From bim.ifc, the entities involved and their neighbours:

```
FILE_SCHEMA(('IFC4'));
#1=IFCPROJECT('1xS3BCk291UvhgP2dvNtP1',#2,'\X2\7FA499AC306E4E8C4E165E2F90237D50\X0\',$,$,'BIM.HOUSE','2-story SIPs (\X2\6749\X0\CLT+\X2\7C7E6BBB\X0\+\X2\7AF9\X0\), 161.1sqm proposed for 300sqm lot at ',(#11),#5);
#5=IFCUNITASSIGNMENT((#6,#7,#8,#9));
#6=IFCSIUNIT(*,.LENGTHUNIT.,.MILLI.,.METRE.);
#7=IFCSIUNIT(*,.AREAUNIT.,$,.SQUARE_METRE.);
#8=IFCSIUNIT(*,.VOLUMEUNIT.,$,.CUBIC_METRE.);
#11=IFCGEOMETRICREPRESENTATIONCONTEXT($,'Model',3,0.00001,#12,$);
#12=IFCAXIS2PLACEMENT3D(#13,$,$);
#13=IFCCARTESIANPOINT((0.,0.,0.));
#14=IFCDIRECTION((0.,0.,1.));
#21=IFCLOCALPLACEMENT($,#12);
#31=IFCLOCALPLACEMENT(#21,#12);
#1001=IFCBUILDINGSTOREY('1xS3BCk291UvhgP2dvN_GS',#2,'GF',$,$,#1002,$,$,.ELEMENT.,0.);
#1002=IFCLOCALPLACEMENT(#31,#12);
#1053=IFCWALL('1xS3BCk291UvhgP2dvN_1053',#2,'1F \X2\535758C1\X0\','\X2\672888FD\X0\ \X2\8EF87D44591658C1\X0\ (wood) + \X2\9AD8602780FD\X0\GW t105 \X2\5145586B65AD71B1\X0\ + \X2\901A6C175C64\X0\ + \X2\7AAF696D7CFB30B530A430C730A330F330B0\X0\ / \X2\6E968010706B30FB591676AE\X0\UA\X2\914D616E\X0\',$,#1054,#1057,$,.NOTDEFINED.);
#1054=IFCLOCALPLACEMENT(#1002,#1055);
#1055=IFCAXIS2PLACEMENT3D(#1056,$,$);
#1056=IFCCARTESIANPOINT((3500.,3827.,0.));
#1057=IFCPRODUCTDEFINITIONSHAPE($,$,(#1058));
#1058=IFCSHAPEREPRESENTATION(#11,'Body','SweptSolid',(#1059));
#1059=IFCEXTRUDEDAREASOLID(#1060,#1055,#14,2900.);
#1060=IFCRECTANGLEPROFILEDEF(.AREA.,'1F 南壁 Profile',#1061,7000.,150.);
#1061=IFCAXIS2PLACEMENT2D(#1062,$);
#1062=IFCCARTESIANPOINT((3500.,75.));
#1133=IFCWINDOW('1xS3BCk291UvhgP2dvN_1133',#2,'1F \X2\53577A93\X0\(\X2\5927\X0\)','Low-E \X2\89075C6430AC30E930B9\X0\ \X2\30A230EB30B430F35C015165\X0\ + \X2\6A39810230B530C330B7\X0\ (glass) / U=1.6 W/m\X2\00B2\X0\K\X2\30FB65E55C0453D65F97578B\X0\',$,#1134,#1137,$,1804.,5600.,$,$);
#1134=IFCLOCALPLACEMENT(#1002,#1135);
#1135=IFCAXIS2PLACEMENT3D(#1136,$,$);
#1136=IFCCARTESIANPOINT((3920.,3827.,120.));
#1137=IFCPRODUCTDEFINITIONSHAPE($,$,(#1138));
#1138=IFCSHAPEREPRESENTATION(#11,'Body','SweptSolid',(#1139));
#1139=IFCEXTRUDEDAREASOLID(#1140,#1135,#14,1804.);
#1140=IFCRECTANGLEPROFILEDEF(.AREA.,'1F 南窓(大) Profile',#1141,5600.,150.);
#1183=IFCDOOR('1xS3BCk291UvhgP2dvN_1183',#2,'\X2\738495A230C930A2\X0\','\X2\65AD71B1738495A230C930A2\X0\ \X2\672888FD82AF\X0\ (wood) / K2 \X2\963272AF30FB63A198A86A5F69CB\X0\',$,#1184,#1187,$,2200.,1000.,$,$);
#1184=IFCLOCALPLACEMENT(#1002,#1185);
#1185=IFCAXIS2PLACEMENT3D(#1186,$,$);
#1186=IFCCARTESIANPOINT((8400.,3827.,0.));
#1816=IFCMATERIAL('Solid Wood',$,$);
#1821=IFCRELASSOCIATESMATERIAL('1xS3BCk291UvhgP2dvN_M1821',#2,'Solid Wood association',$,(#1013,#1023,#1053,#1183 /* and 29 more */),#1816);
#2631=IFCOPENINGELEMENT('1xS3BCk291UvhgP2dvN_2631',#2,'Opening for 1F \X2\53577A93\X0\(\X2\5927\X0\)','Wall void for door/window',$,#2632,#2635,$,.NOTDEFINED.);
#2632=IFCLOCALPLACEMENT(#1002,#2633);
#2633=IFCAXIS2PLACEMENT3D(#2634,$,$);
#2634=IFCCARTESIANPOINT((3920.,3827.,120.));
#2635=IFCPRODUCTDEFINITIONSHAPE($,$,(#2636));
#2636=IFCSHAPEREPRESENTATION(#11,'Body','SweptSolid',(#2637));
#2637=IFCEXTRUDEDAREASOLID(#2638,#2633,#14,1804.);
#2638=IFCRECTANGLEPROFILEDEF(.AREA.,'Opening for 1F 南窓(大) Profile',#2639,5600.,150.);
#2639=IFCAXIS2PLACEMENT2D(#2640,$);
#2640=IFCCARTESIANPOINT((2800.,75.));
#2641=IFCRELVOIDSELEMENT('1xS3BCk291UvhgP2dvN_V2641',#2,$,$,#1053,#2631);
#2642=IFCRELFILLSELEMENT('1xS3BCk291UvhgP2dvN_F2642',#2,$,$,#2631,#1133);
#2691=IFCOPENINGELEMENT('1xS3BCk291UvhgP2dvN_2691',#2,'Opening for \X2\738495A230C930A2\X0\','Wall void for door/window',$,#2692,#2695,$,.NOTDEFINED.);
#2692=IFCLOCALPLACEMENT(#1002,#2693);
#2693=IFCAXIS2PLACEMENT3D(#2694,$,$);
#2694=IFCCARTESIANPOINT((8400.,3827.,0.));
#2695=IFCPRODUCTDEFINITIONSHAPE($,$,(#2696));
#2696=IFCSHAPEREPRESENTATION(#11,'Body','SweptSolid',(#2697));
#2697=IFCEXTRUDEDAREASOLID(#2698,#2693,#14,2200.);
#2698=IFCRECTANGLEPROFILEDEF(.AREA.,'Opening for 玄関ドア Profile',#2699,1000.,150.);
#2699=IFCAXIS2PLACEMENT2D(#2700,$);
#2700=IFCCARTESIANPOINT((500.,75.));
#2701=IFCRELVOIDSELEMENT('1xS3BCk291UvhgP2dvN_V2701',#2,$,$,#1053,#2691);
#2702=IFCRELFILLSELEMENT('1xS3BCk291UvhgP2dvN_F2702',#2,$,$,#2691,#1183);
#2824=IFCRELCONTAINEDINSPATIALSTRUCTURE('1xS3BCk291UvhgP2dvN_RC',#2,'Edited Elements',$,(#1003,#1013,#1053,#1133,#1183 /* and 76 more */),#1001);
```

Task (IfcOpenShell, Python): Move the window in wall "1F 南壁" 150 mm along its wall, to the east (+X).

```python
import ifcopenshell
import ifcopenshell.api.geometry
import ifcopenshell.util.placement
import ifcopenshell.util.unit

model = ifcopenshell.open("bim.ifc")
unit_scale = ifcopenshell.util.unit.calculate_unit_scale(model)

window = model.by_guid("1xS3BCk291UvhgP2dvN_1133")
opening = window.FillsVoids[0].RelatingOpeningElement
wall = opening.VoidsElements[0].RelatingBuildingElement

wall_matrix = ifcopenshell.util.placement.get_local_placement(wall.ObjectPlacement)
shift = wall_matrix[:3, 0] * 0.15 / unit_scale
before = ifcopenshell.util.placement.get_local_placement(window.ObjectPlacement)[:3, 3].copy()

# The window is not placed relative to its opening, so move both.
for product in (opening, window):
    matrix = ifcopenshell.util.placement.get_local_placement(product.ObjectPlacement)
    matrix[:3, 3] += shift
    ifcopenshell.api.geometry.edit_object_placement(model, product=product, matrix=matrix, is_si=False)

after = ifcopenshell.util.placement.get_local_placement(window.ObjectPlacement)[:3, 3]
print("window moved by", (after - before).round(3) + 0.0)

model.write("bim_updated.ifc")
```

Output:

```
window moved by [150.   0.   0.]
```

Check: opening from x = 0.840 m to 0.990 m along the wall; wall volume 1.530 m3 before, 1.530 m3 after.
